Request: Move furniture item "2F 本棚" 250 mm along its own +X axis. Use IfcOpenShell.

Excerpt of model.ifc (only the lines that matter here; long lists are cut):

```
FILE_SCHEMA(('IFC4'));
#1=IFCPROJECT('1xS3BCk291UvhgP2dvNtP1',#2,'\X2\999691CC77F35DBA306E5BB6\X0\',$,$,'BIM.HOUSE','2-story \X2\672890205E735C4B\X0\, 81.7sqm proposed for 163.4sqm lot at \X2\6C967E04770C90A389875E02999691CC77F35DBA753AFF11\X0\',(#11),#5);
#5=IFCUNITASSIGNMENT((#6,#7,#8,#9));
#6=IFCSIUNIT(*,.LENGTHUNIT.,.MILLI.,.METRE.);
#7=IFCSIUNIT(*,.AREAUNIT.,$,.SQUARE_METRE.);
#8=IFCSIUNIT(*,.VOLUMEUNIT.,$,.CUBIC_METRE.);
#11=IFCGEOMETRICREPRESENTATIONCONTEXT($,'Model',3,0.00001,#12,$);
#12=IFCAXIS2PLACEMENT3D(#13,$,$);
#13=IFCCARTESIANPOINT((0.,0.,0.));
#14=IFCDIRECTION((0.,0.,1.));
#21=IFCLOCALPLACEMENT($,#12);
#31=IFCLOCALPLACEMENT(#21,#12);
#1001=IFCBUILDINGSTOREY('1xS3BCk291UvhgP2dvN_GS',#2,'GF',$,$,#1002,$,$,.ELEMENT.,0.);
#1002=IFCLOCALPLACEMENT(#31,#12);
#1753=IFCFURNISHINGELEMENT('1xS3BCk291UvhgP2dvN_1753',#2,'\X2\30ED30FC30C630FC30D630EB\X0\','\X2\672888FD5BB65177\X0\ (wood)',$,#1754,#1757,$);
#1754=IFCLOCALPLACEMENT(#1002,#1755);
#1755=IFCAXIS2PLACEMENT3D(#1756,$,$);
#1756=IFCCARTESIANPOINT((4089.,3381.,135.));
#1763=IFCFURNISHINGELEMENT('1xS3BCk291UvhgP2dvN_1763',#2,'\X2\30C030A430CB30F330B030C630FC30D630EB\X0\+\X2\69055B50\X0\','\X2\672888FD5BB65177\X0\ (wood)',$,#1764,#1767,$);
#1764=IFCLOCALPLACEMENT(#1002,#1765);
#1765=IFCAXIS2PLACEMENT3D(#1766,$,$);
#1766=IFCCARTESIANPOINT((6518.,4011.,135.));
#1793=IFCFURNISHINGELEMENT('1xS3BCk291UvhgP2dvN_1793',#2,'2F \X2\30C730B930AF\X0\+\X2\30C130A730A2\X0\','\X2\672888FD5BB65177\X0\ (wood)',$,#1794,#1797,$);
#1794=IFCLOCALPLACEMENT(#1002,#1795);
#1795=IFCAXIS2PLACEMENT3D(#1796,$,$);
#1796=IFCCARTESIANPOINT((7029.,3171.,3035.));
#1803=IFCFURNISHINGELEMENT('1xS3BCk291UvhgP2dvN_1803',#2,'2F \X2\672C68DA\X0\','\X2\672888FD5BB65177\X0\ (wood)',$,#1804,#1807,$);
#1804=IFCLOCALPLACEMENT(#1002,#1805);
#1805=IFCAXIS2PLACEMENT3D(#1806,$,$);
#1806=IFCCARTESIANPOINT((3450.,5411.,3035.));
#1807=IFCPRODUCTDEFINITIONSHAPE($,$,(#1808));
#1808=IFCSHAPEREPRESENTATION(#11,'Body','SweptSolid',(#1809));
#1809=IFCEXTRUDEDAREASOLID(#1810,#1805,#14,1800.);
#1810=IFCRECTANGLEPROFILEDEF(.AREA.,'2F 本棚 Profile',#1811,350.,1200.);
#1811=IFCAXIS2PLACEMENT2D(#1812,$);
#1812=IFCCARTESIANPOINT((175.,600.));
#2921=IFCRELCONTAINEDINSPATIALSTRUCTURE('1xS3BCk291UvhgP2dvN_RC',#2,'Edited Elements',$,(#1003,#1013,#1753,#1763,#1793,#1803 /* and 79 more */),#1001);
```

```python
import ifcopenshell
import ifcopenshell.api.geometry
import ifcopenshell.util.placement

model = ifcopenshell.open("model.ifc")

item = model.by_guid("1xS3BCk291UvhgP2dvN_1803")
matrix = ifcopenshell.util.placement.get_local_placement(item.ObjectPlacement)
matrix[:3, 3] += matrix[:3, 0] * 250.0
ifcopenshell.api.geometry.edit_object_placement(model, product=item, matrix=matrix, is_si=False)

print(ifcopenshell.util.placement.get_local_placement(item.ObjectPlacement).round(3) + 0.0)

model.write("model-out.ifc")
```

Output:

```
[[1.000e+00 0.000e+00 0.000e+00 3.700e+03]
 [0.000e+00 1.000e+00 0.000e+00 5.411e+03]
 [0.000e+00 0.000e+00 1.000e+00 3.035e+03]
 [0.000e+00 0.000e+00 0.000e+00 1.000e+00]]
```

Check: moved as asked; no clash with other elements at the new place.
